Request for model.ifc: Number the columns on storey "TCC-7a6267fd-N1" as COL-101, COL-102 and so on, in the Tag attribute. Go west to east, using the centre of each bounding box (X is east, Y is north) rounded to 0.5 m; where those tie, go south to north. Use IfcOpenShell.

First a look at what the model holds.

```python
import ifcopenshell
import ifcopenshell.util.element
import ifcopenshell.util.placement

model = ifcopenshell.open("model.ifc")
print(model.schema)
storey = next(s for s in model.by_type("IfcBuildingStorey") if s.Name == "TCC-7a6267fd-N1")
columns = [e for e in ifcopenshell.util.element.get_decomposition(storey) if e.is_a("IfcColumn")]
for e in sorted(columns, key=lambda e: e.id()):
    origin = ifcopenshell.util.placement.get_local_placement(e.ObjectPlacement)[:3, 3]
    print(e.id(), e.Tag, e.Name, origin.round(2) + 0.0, sep=" | ")
```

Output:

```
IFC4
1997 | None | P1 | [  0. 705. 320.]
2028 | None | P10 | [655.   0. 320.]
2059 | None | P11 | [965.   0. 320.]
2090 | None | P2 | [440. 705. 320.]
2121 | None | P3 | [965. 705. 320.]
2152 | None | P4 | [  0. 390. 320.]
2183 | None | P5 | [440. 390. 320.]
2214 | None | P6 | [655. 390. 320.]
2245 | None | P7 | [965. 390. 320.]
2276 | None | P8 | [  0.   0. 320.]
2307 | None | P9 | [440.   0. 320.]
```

```python
import ifcopenshell
import ifcopenshell.geom
import ifcopenshell.util.element
import ifcopenshell.util.shape

model = ifcopenshell.open("model.ifc")
settings = ifcopenshell.geom.settings()
settings.set("use-world-coords", True)


def centre(element):
    shape = ifcopenshell.geom.create_shape(settings, element)
    return ifcopenshell.util.shape.get_bbox_centroid(shape.geometry)


storey = next(s for s in model.by_type("IfcBuildingStorey") if s.Name == "TCC-7a6267fd-N1")
columns = [e for e in ifcopenshell.util.element.get_decomposition(storey) if e.is_a("IfcColumn")]

# Insertion points can sit at a corner or the storey origin, so sort by the geometry (in metres).
centres = {e: centre(e) for e in columns}
columns.sort(key=lambda e: (round(centres[e][0] / 0.5), centres[e][1]))

for i, e in enumerate(columns, start=1):
    number = f"COL-1{i:02d}"
    e.Tag = number
    print(e.id(), number)

model.write("model_v2.ifc")
```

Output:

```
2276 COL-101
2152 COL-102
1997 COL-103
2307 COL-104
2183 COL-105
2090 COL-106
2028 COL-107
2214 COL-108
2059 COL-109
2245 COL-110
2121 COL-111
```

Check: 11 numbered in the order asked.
